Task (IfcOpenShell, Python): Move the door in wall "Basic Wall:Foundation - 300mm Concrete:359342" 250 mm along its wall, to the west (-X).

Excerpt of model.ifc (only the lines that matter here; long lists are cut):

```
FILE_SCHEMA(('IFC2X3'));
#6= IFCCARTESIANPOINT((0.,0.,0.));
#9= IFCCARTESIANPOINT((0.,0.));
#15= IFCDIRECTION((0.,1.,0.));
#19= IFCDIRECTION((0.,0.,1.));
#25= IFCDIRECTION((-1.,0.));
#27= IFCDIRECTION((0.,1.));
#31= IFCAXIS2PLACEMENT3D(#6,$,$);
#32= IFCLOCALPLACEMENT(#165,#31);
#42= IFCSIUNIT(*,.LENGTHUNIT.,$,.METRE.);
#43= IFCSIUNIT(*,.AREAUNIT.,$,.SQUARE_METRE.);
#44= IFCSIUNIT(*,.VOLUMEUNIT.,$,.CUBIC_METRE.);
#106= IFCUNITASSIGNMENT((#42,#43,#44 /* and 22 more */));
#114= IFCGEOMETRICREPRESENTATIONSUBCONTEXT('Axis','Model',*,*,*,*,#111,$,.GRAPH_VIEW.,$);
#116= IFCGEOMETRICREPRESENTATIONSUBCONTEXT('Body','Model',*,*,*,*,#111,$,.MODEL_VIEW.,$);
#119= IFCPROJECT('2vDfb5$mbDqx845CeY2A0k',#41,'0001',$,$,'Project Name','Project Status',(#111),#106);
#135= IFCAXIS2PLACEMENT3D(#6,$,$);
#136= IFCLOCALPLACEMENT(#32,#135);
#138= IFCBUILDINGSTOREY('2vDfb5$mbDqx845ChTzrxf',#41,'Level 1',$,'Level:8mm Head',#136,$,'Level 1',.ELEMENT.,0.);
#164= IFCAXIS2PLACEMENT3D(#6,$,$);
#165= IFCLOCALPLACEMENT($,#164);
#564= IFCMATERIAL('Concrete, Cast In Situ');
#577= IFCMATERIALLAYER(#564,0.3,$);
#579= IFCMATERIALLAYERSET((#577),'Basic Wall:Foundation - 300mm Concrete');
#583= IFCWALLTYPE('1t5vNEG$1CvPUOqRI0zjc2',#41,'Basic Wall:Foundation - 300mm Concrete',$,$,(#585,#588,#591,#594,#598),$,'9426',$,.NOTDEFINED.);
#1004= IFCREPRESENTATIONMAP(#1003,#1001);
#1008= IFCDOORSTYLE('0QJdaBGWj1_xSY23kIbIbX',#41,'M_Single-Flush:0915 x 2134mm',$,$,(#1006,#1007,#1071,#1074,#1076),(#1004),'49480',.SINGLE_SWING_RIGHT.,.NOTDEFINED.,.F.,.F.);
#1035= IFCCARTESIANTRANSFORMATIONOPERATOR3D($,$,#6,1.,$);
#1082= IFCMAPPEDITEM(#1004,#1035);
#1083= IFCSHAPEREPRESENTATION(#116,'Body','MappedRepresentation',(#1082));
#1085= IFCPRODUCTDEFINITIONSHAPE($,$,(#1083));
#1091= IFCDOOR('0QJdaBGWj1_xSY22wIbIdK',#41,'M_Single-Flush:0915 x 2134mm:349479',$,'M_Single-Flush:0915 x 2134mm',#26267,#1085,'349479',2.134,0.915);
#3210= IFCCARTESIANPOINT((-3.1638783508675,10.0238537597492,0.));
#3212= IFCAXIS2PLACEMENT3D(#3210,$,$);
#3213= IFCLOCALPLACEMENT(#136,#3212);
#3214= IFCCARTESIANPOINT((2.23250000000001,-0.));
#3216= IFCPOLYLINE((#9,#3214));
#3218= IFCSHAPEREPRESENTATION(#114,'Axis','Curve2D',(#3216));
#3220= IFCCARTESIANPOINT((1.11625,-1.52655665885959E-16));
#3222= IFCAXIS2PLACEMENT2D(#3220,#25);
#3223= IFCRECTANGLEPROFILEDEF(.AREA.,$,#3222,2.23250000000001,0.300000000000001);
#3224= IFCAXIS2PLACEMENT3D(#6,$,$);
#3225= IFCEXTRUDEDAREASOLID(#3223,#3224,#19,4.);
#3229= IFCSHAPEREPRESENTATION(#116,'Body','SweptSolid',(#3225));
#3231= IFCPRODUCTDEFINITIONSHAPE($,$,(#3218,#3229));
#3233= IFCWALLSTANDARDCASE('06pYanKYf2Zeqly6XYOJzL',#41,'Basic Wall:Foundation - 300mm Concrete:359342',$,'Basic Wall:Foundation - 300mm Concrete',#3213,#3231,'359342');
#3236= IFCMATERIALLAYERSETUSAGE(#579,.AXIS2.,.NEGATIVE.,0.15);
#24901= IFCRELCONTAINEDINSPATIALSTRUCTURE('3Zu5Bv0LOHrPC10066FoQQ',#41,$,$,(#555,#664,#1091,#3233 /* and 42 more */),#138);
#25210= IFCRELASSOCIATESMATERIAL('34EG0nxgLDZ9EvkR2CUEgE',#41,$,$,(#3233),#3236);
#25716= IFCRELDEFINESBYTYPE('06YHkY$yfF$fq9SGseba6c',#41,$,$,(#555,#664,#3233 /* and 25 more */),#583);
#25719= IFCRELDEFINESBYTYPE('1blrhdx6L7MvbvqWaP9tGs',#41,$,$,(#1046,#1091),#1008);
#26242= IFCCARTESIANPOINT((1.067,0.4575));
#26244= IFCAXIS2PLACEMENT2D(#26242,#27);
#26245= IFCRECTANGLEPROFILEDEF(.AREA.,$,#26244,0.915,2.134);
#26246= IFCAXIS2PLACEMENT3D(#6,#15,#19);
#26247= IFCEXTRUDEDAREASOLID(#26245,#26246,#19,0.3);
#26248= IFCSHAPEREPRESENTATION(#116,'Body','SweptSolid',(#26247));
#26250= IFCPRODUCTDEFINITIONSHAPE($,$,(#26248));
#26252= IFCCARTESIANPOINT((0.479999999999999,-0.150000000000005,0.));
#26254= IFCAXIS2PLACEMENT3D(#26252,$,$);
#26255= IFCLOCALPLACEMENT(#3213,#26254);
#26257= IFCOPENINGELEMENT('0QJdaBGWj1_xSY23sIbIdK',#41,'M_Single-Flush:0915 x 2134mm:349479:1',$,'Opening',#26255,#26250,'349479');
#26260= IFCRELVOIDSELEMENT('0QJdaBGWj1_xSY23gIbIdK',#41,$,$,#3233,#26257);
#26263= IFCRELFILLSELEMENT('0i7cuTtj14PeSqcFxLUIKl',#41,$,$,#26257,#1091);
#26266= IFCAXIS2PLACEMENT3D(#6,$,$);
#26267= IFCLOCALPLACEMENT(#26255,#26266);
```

```python
import ifcopenshell
import ifcopenshell.api.geometry
import ifcopenshell.util.placement

model = ifcopenshell.open("model.ifc")

door = model.by_id(1091)
opening = door.FillsVoids[0].RelatingOpeningElement
wall = opening.VoidsElements[0].RelatingBuildingElement

wall_matrix = ifcopenshell.util.placement.get_local_placement(wall.ObjectPlacement)
shift = wall_matrix[:3, 0] * -0.25
before = ifcopenshell.util.placement.get_local_placement(door.ObjectPlacement)[:3, 3].copy()

# The door is placed relative to its opening, so it follows when the opening moves.
matrix = ifcopenshell.util.placement.get_local_placement(opening.ObjectPlacement)
matrix[:3, 3] += shift
ifcopenshell.api.geometry.edit_object_placement(
    model, product=opening, matrix=matrix, is_si=False, should_transform_children=True
)

after = ifcopenshell.util.placement.get_local_placement(door.ObjectPlacement)[:3, 3]
print("door moved by", (after - before).round(3) + 0.0)

model.write("model_rev.ifc")
```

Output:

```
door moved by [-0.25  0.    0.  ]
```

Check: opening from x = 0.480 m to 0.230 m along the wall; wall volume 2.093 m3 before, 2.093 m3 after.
